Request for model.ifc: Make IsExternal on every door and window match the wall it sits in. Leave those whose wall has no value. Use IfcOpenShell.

First a look at what the model holds.

```python
import ifcopenshell
import ifcopenshell.util.element

model = ifcopenshell.open("model.ifc")
print(model.schema)
seen = {}
for e in model.by_type("IfcDoor") + model.by_type("IfcWindow"):
    if not e.FillsVoids:
        continue
    host = e.FillsVoids[0].RelatingOpeningElement.VoidsElements[0].RelatingBuildingElement
    own = ifcopenshell.util.element.get_pset(e, f"Pset_{e.is_a()[3:].removesuffix('StandardCase')}Common", "IsExternal")
    wall = ifcopenshell.util.element.get_pset(host, "Pset_WallCommon", "IsExternal")
    seen[e.is_a(), own, wall] = seen.get((e.is_a(), own, wall), 0) + 1
for (cls, own, wall), count in sorted(seen.items(), key=str):
    print(count, cls, "IsExternal:", own, "| host wall:", wall)
```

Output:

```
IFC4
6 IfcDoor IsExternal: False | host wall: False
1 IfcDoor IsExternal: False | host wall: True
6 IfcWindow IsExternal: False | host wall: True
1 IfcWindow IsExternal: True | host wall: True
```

```python
import ifcopenshell
import ifcopenshell.api.pset
import ifcopenshell.util.element

model = ifcopenshell.open("model.ifc")

count = 0
for ifc_class, pset_name in (("IfcDoor", "Pset_DoorCommon"), ("IfcWindow", "Pset_WindowCommon")):
    for e in model.by_type(ifc_class):
        if not e.FillsVoids:
            continue
        host = e.FillsVoids[0].RelatingOpeningElement.VoidsElements[0].RelatingBuildingElement
        external = ifcopenshell.util.element.get_pset(host, "Pset_WallCommon", "IsExternal")
        if external is None or ifcopenshell.util.element.get_pset(e, pset_name, "IsExternal") == external:
            continue
        pset = ifcopenshell.api.pset.add_pset(model, product=e, name=pset_name)
        ifcopenshell.api.pset.edit_pset(model, pset=pset, properties={"IsExternal": external})
        count += 1

print(count, "updated")

model.write("model-out.ifc")
```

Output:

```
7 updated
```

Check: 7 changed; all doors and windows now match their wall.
